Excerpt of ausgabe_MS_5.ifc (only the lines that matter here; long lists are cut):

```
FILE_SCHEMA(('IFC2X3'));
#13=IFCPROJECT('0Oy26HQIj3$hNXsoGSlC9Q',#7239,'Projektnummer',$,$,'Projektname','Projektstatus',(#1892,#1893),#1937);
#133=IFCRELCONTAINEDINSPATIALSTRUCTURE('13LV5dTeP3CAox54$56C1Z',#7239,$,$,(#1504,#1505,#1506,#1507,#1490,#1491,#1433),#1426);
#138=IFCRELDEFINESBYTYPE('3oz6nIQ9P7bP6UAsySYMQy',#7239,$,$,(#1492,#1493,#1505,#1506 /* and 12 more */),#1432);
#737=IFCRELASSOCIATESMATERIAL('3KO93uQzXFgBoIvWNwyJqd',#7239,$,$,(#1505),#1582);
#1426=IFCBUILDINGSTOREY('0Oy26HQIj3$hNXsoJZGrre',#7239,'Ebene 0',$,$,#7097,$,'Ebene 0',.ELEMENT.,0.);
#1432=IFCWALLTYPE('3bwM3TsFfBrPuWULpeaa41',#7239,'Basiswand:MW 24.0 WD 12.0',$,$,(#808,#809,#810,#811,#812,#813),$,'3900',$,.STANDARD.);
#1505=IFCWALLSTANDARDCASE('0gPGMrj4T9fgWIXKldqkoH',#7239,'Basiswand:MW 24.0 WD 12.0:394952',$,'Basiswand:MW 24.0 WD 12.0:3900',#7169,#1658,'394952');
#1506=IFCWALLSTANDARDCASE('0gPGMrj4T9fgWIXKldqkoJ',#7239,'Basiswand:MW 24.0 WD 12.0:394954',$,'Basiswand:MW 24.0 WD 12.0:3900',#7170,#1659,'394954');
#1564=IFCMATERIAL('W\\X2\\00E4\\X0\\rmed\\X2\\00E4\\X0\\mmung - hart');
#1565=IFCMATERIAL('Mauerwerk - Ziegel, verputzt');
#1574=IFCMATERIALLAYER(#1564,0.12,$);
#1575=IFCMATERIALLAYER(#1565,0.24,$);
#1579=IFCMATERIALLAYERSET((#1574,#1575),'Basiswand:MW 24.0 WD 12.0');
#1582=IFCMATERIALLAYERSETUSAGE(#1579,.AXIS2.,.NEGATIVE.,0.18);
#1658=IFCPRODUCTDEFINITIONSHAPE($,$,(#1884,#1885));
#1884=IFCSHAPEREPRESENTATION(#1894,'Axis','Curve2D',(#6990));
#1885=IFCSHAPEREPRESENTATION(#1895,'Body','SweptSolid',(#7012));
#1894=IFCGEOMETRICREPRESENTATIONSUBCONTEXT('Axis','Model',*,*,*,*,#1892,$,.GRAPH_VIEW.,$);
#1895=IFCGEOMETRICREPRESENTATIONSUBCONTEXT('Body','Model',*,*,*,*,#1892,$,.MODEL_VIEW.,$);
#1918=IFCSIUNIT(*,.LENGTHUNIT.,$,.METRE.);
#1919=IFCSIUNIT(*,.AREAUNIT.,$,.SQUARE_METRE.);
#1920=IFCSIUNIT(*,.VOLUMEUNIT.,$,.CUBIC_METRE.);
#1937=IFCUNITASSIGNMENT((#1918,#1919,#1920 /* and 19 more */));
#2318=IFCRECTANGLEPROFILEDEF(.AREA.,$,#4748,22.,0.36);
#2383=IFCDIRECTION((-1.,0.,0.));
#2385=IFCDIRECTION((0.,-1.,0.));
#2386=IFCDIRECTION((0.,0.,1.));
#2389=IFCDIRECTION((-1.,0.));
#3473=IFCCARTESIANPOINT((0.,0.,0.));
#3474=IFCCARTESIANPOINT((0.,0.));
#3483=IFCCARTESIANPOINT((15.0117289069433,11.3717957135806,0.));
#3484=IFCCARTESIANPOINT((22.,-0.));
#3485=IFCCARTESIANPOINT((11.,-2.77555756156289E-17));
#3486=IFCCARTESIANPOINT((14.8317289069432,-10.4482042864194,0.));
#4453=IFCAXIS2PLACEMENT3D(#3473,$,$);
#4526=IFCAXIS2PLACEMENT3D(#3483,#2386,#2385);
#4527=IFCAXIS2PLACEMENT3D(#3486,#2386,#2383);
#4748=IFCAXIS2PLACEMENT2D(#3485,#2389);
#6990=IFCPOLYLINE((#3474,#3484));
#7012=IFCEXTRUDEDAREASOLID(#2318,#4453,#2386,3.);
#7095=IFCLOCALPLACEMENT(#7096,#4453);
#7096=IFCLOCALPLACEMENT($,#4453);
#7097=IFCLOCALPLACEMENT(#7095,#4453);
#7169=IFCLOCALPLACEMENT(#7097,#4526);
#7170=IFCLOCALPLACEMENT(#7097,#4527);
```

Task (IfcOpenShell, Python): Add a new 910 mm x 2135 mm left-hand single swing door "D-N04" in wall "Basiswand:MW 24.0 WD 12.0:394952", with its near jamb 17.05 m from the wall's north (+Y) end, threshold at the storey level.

```python
import numpy as np
import ifcopenshell
import ifcopenshell.api.feature
import ifcopenshell.api.geometry
import ifcopenshell.api.root
import ifcopenshell.api.spatial
import ifcopenshell.api.type
import ifcopenshell.geom
import ifcopenshell.util.element
import ifcopenshell.util.placement
import ifcopenshell.util.representation
import ifcopenshell.util.shape
import ifcopenshell.util.unit

model = ifcopenshell.open("ausgabe_MS_5.ifc")
unit_scale = ifcopenshell.util.unit.calculate_unit_scale(model)
settings = ifcopenshell.geom.settings()


def volume(element):
    """Net volume in cubic metres, openings subtracted."""
    shape = ifcopenshell.geom.create_shape(settings, element)
    return ifcopenshell.util.shape.get_volume(shape.geometry)


wall = model.by_guid("0gPGMrj4T9fgWIXKldqkoH")
storey = ifcopenshell.util.element.get_container(wall, ifc_class="IfcBuildingStorey")
context = ifcopenshell.util.representation.get_context(model, "Model", "Body", "MODEL_VIEW")
before = volume(wall)

width, height, from_end, sill = 0.91, 2.135, 17.05, 0.0  # metres

# The wall runs along its own X axis, and the end named is its -X end.
wall_shape = ifcopenshell.geom.create_shape(settings, wall)
x, y, z = ifcopenshell.util.shape.get_vertices(wall_shape.geometry).T
start = x.min() + from_end
face, thickness = float(y.min()), float(y.max() - y.min())
wall_matrix = ifcopenshell.util.placement.get_local_placement(wall.ObjectPlacement)
level = ifcopenshell.util.placement.get_local_placement(storey.ObjectPlacement)[2, 3]


def in_wall(x, y):
    """Placement at x, y metres in the wall's axes, at sill height."""
    matrix = wall_matrix.copy()
    matrix[:, 3] = wall_matrix @ np.array([x / unit_scale, y / unit_scale, 0.0, 1.0])
    matrix[2, 3] = level + sill / unit_scale
    return matrix


# Opening: a box that overshoots both wall faces by 50 mm.
opening = ifcopenshell.api.root.create_entity(model, ifc_class="IfcOpeningElement")
box = ifcopenshell.api.geometry.add_wall_representation(
    model, context=context, length=width, height=height, thickness=thickness + 0.1
)
ifcopenshell.api.geometry.assign_representation(model, product=opening, representation=box)
ifcopenshell.api.geometry.edit_object_placement(model, product=opening, matrix=in_wall(start, face - 0.05), is_si=False)
ifcopenshell.api.feature.add_feature(model, feature=opening, element=wall)

door = ifcopenshell.api.root.create_entity(model, ifc_class="IfcDoor", name="D-N04")
door.OverallWidth, door.OverallHeight = width / unit_scale, height / unit_scale
body = ifcopenshell.api.geometry.add_door_representation(
    model,
    context=context,
    overall_width=door.OverallWidth,
    overall_height=door.OverallHeight,
    operation_type="SINGLE_SWING_LEFT",
    lining_properties={"LiningDepth": thickness / unit_scale, "ThresholdDepth": thickness / unit_scale},
)
ifcopenshell.api.geometry.assign_representation(model, product=door, representation=body)
ifcopenshell.api.spatial.assign_container(model, products=[door], relating_structure=storey)
fills = ifcopenshell.api.feature.add_filling(model, opening=opening, element=door)
fills.OwnerHistory = door.OwnerHistory  # required in IFC2X3

# IFC2X3 keeps the operation on the door style.
style = ifcopenshell.api.root.create_entity(model, ifc_class="IfcDoorStyle", name="D-N04")
style.OperationType, style.ConstructionType = "SINGLE_SWING_LEFT", "NOTDEFINED"
style.ParameterTakesPrecedence = style.Sizeable = False
ifcopenshell.api.type.assign_type(model, related_objects=[door], relating_type=style)

# The lining spans the wall, so the door starts at the wall face.
ifcopenshell.api.geometry.edit_object_placement(model, product=door, matrix=in_wall(start, face), is_si=False)

after = volume(wall)

print(f"wall volume {before:.3f} -> {after:.3f} m3")

model.write("ausgabe_MS_5_updated.ifc")
```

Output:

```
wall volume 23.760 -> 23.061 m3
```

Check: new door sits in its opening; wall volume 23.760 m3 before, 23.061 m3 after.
